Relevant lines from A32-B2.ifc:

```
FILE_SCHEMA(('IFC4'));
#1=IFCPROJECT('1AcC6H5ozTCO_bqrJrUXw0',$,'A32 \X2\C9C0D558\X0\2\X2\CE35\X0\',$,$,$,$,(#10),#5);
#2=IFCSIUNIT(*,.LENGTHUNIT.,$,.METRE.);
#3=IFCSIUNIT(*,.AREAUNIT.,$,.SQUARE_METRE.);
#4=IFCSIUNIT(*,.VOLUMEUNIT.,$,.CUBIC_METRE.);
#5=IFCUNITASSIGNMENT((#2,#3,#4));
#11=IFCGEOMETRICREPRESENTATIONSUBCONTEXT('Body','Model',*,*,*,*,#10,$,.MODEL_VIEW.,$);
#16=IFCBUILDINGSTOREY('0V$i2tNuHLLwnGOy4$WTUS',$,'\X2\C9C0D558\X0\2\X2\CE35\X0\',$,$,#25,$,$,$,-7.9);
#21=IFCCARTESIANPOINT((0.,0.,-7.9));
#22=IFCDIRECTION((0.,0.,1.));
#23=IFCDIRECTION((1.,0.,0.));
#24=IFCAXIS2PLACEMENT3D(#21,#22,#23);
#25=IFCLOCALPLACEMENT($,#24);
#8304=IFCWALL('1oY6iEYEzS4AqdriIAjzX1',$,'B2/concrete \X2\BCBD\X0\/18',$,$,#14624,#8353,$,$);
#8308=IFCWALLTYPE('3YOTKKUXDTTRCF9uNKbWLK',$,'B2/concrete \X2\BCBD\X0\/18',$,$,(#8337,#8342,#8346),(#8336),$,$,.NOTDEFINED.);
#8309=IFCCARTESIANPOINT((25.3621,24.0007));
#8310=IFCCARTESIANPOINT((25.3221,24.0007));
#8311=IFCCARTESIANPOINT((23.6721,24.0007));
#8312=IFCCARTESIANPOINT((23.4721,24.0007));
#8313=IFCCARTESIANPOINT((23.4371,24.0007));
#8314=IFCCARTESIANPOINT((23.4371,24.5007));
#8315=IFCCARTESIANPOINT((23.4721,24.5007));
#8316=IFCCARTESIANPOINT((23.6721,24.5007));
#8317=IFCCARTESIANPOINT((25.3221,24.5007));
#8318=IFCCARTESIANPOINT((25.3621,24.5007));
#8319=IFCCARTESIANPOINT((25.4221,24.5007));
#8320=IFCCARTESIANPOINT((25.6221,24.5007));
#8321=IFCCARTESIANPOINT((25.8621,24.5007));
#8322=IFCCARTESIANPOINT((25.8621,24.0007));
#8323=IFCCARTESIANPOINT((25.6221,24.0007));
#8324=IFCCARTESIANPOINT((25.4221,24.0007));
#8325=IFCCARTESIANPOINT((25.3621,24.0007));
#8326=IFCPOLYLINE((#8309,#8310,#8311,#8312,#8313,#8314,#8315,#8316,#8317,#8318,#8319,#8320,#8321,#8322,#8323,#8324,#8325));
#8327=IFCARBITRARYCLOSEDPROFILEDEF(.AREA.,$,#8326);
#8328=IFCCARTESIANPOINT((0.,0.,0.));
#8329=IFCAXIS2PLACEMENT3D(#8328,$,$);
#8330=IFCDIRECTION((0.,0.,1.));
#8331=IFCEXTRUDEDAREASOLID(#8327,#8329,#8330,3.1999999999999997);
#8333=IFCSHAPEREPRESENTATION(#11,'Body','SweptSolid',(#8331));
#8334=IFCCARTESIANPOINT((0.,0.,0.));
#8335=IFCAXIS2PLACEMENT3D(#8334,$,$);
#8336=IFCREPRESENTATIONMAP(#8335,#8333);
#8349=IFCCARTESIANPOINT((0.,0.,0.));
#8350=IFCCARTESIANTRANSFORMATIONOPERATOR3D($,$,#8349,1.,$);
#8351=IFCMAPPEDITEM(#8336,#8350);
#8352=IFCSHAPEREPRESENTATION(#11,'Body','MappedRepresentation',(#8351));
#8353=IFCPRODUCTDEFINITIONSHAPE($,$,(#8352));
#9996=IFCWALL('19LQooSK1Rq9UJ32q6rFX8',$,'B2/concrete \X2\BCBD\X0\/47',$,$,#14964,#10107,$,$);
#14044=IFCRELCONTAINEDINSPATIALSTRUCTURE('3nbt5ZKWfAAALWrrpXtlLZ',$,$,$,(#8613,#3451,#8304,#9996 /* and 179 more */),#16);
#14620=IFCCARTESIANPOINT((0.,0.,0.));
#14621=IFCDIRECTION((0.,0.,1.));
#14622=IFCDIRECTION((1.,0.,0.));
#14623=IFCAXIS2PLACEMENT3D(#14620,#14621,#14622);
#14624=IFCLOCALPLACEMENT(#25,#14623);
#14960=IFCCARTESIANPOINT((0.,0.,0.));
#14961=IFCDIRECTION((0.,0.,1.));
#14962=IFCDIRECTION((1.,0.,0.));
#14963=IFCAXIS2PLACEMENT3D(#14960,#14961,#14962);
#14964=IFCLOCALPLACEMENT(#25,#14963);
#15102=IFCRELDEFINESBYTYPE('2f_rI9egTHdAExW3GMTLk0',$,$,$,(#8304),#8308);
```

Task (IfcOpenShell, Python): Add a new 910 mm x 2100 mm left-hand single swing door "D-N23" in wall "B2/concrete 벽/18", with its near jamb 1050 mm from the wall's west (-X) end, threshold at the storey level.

```python
import numpy as np
import ifcopenshell
import ifcopenshell.api.feature
import ifcopenshell.api.geometry
import ifcopenshell.api.root
import ifcopenshell.api.spatial
import ifcopenshell.geom
import ifcopenshell.util.element
import ifcopenshell.util.placement
import ifcopenshell.util.representation
import ifcopenshell.util.shape
import ifcopenshell.util.unit

model = ifcopenshell.open("A32-B2.ifc")
unit_scale = ifcopenshell.util.unit.calculate_unit_scale(model)
settings = ifcopenshell.geom.settings()


def volume(element):
    """Net volume in cubic metres, openings subtracted."""
    shape = ifcopenshell.geom.create_shape(settings, element)
    return ifcopenshell.util.shape.get_volume(shape.geometry)


wall = model.by_guid("1oY6iEYEzS4AqdriIAjzX1")
storey = ifcopenshell.util.element.get_container(wall, ifc_class="IfcBuildingStorey")
context = ifcopenshell.util.representation.get_context(model, "Model", "Body", "MODEL_VIEW")
before = volume(wall)

width, height, from_end, sill = 0.91, 2.1, 1.05, 0.0  # metres

# The wall runs along its own X axis, and the end named is its -X end.
wall_shape = ifcopenshell.geom.create_shape(settings, wall)
x, y, z = ifcopenshell.util.shape.get_vertices(wall_shape.geometry).T
start = x.min() + from_end
face, thickness = float(y.min()), float(y.max() - y.min())
wall_matrix = ifcopenshell.util.placement.get_local_placement(wall.ObjectPlacement)
level = ifcopenshell.util.placement.get_local_placement(storey.ObjectPlacement)[2, 3]


def in_wall(x, y):
    """Placement at x, y metres in the wall's axes, at sill height."""
    matrix = wall_matrix.copy()
    matrix[:, 3] = wall_matrix @ np.array([x / unit_scale, y / unit_scale, 0.0, 1.0])
    matrix[2, 3] = level + sill / unit_scale
    return matrix


# Opening: a box that overshoots both wall faces by 50 mm.
opening = ifcopenshell.api.root.create_entity(model, ifc_class="IfcOpeningElement", predefined_type="OPENING")
box = ifcopenshell.api.geometry.add_wall_representation(
    model, context=context, length=width, height=height, thickness=thickness + 0.1
)
ifcopenshell.api.geometry.assign_representation(model, product=opening, representation=box)
ifcopenshell.api.geometry.edit_object_placement(model, product=opening, matrix=in_wall(start, face - 0.05), is_si=False)
ifcopenshell.api.feature.add_feature(model, feature=opening, element=wall)

door = ifcopenshell.api.root.create_entity(model, ifc_class="IfcDoor", name="D-N23", predefined_type="DOOR")
door.OverallWidth, door.OverallHeight = width / unit_scale, height / unit_scale
door.OperationType = "SINGLE_SWING_LEFT"
body = ifcopenshell.api.geometry.add_door_representation(
    model,
    context=context,
    overall_width=door.OverallWidth,
    overall_height=door.OverallHeight,
    operation_type="SINGLE_SWING_LEFT",
    lining_properties={"LiningDepth": thickness / unit_scale, "ThresholdDepth": thickness / unit_scale},
)
ifcopenshell.api.geometry.assign_representation(model, product=door, representation=body)
ifcopenshell.api.spatial.assign_container(model, products=[door], relating_structure=storey)
ifcopenshell.api.feature.add_filling(model, opening=opening, element=door)

# The lining spans the wall, so the door starts at the wall face.
ifcopenshell.api.geometry.edit_object_placement(model, product=door, matrix=in_wall(start, face), is_si=False)

after = volume(wall)

print(f"wall volume {before:.3f} -> {after:.3f} m3")

model.write("A32-B2_v2.ifc")
```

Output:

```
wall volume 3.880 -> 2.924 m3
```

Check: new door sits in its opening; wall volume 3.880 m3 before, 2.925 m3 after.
